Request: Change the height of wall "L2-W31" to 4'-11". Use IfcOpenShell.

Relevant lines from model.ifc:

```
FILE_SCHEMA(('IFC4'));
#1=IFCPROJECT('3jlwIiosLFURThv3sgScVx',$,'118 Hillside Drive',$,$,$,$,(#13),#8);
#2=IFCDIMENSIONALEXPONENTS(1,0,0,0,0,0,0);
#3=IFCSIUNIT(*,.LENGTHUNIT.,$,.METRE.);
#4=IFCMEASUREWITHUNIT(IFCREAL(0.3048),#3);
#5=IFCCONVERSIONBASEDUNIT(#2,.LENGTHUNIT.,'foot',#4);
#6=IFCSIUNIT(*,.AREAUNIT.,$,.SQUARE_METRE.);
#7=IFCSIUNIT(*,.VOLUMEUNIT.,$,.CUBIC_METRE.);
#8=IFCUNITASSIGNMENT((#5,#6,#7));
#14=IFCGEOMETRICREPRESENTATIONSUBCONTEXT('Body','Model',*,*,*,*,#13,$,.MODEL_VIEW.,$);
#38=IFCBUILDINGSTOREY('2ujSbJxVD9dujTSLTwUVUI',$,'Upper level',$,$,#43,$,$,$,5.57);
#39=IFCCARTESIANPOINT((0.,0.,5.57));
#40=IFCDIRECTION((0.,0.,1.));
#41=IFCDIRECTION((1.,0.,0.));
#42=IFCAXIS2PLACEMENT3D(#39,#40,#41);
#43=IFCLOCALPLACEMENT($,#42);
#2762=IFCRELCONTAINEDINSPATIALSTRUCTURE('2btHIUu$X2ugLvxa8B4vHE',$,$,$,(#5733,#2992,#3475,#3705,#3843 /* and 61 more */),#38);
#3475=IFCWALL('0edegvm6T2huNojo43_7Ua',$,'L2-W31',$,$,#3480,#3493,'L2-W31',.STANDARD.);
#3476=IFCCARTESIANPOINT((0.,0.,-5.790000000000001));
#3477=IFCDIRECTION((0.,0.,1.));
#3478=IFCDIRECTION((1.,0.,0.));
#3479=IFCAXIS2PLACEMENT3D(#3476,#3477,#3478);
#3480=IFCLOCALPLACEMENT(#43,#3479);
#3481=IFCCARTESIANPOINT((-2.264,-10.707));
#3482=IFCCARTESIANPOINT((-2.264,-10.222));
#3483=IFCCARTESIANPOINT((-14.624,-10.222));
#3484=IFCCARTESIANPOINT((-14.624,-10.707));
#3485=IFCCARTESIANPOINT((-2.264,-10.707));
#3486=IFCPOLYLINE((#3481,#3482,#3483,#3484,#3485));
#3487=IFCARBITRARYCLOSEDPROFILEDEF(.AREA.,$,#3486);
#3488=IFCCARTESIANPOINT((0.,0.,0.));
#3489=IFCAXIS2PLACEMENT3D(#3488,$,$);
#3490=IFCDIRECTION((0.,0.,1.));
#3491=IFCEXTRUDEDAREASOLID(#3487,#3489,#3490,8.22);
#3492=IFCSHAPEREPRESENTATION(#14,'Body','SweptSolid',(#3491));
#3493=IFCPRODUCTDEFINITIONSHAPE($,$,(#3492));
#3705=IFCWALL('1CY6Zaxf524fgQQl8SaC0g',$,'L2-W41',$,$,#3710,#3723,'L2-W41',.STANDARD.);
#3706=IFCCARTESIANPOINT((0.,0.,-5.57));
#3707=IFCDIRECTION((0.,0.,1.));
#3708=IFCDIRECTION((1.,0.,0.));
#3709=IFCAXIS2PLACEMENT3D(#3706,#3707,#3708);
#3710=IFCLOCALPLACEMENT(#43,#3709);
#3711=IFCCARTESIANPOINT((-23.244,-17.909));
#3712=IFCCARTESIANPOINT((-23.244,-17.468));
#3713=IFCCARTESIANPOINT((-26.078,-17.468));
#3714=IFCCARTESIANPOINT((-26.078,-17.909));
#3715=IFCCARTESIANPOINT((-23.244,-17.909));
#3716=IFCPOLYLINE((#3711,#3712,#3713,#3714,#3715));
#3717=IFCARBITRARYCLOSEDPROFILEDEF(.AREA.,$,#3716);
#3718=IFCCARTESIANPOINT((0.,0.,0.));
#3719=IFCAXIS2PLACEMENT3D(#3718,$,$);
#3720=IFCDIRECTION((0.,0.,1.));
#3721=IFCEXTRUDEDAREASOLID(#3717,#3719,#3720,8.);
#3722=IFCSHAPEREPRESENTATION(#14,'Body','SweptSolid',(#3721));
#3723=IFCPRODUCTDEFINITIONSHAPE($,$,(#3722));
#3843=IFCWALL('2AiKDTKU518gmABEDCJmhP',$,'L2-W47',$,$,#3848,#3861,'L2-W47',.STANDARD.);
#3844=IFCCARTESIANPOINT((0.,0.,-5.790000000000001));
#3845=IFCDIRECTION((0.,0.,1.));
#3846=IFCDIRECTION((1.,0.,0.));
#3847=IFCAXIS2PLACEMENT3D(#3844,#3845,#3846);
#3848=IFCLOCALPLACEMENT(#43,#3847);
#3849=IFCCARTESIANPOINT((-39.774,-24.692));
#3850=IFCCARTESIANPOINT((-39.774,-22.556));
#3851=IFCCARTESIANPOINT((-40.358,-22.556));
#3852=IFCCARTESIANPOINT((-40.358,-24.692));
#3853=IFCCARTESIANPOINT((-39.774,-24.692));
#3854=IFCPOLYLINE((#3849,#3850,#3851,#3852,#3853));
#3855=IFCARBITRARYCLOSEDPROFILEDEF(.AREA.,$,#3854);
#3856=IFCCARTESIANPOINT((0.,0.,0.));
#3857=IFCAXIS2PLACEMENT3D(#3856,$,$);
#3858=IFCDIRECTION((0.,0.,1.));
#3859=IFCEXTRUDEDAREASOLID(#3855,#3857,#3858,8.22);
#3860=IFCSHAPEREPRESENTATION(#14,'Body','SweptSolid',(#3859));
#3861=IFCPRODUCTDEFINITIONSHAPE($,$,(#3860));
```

```python
import ifcopenshell
import ifcopenshell.geom
import ifcopenshell.util.representation
import ifcopenshell.util.shape
import ifcopenshell.util.unit

model = ifcopenshell.open("model.ifc")
unit_scale = ifcopenshell.util.unit.calculate_unit_scale(model)
settings = ifcopenshell.geom.settings()


def volume(element):
    """Net volume in cubic metres, openings subtracted."""
    shape = ifcopenshell.geom.create_shape(settings, element)
    return ifcopenshell.util.shape.get_volume(shape.geometry)


wall = model.by_guid("0edegvm6T2huNojo43_7Ua")
before = volume(wall)

body = ifcopenshell.util.representation.get_representation(wall, "Model", "Body")
solid = body.Items[0]
old_height = solid.Depth
solid.Depth = 59 * 0.0254 / unit_scale
after = volume(wall)

print(f"height {old_height:g} -> {solid.Depth:g}, volume {before:.3f} -> {after:.3f} m3")

model.write("model_updated.ifc")
```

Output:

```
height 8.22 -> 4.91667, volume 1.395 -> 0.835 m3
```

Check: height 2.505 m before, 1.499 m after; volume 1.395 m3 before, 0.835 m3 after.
